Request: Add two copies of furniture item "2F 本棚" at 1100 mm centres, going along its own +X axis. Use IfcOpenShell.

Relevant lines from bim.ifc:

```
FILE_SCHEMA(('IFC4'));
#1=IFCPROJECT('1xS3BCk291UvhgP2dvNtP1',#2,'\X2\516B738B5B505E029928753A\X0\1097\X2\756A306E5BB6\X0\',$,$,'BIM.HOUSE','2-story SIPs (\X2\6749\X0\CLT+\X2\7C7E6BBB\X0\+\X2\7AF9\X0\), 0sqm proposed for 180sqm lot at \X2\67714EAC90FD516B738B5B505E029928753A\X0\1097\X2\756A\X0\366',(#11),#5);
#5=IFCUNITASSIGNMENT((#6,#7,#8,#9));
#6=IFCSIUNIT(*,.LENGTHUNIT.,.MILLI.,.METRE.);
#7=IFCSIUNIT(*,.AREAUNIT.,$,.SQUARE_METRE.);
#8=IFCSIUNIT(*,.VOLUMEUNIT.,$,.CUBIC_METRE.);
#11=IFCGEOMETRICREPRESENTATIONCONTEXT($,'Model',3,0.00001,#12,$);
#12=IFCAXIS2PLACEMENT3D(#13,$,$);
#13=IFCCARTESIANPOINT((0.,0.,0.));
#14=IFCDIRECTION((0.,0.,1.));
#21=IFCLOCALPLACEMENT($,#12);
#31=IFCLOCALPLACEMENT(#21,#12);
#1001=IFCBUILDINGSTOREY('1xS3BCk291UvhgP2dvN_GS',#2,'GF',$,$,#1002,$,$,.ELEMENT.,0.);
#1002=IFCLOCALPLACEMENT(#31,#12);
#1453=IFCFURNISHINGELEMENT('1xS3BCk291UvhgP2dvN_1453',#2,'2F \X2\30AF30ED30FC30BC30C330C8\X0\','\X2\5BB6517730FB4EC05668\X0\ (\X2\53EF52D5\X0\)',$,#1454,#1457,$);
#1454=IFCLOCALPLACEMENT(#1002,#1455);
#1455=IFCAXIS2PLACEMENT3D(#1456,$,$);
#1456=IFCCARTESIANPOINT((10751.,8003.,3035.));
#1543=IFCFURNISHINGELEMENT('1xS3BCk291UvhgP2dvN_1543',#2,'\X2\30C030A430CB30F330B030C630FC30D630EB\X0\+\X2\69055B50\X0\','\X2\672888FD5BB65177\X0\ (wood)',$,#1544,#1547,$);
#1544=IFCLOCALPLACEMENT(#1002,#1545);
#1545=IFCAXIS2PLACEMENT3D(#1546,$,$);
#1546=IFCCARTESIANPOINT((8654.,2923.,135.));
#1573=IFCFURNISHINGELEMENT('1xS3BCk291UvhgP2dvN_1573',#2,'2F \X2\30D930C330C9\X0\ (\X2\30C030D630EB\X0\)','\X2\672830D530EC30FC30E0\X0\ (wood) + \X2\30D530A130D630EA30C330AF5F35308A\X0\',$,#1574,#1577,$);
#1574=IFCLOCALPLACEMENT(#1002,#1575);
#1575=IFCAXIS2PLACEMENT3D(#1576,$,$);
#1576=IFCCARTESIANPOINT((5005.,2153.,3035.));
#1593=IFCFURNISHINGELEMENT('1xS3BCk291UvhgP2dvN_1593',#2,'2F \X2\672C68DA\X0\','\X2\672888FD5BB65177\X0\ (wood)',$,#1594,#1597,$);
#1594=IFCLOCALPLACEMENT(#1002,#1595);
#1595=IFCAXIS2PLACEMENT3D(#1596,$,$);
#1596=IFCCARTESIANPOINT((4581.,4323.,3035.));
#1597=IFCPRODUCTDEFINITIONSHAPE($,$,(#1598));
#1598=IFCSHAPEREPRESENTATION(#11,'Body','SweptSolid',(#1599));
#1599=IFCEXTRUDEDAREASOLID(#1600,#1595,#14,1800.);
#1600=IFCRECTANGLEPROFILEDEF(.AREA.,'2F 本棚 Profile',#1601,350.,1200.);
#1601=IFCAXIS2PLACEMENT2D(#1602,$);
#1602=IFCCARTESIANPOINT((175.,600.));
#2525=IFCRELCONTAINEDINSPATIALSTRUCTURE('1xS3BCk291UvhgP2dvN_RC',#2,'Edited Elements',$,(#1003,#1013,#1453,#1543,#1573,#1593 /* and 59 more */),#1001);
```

```python
import ifcopenshell
import ifcopenshell.api.geometry
import ifcopenshell.api.root
import ifcopenshell.util.element
import ifcopenshell.util.placement

model = ifcopenshell.open("bim.ifc")


def reuse_history(source, copy):
    """copy_class also copies each property set's owner history, people and application; keep the originals."""
    for rel in copy.IsDefinedBy:
        if rel.is_a("IfcRelDefinesByProperties") and (history := rel.RelatingPropertyDefinition.OwnerHistory):
            rel.RelatingPropertyDefinition.OwnerHistory = source.OwnerHistory
            ifcopenshell.util.element.remove_deep2(model, history)


source = model.by_guid("1xS3BCk291UvhgP2dvN_1593")
base = ifcopenshell.util.placement.get_local_placement(source.ObjectPlacement)
step = base[:3, 0] * 1100.0

for i in range(1, 3):
    copy = ifcopenshell.api.root.copy_class(model, product=source)
    copy.Representation = ifcopenshell.util.element.copy_deep(
        model, source.Representation, exclude=["IfcGeometricRepresentationContext", "IfcRepresentationMap"]
    )
    reuse_history(source, copy)
    matrix = base.copy()
    matrix[:3, 3] += i * step
    print("added at", matrix[:3, 3].round(3) + 0.0)
    ifcopenshell.api.geometry.edit_object_placement(model, product=copy, matrix=matrix, is_si=False)

model.write("bim_rev.ifc")
```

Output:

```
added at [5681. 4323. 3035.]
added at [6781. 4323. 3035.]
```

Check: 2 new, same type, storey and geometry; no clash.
